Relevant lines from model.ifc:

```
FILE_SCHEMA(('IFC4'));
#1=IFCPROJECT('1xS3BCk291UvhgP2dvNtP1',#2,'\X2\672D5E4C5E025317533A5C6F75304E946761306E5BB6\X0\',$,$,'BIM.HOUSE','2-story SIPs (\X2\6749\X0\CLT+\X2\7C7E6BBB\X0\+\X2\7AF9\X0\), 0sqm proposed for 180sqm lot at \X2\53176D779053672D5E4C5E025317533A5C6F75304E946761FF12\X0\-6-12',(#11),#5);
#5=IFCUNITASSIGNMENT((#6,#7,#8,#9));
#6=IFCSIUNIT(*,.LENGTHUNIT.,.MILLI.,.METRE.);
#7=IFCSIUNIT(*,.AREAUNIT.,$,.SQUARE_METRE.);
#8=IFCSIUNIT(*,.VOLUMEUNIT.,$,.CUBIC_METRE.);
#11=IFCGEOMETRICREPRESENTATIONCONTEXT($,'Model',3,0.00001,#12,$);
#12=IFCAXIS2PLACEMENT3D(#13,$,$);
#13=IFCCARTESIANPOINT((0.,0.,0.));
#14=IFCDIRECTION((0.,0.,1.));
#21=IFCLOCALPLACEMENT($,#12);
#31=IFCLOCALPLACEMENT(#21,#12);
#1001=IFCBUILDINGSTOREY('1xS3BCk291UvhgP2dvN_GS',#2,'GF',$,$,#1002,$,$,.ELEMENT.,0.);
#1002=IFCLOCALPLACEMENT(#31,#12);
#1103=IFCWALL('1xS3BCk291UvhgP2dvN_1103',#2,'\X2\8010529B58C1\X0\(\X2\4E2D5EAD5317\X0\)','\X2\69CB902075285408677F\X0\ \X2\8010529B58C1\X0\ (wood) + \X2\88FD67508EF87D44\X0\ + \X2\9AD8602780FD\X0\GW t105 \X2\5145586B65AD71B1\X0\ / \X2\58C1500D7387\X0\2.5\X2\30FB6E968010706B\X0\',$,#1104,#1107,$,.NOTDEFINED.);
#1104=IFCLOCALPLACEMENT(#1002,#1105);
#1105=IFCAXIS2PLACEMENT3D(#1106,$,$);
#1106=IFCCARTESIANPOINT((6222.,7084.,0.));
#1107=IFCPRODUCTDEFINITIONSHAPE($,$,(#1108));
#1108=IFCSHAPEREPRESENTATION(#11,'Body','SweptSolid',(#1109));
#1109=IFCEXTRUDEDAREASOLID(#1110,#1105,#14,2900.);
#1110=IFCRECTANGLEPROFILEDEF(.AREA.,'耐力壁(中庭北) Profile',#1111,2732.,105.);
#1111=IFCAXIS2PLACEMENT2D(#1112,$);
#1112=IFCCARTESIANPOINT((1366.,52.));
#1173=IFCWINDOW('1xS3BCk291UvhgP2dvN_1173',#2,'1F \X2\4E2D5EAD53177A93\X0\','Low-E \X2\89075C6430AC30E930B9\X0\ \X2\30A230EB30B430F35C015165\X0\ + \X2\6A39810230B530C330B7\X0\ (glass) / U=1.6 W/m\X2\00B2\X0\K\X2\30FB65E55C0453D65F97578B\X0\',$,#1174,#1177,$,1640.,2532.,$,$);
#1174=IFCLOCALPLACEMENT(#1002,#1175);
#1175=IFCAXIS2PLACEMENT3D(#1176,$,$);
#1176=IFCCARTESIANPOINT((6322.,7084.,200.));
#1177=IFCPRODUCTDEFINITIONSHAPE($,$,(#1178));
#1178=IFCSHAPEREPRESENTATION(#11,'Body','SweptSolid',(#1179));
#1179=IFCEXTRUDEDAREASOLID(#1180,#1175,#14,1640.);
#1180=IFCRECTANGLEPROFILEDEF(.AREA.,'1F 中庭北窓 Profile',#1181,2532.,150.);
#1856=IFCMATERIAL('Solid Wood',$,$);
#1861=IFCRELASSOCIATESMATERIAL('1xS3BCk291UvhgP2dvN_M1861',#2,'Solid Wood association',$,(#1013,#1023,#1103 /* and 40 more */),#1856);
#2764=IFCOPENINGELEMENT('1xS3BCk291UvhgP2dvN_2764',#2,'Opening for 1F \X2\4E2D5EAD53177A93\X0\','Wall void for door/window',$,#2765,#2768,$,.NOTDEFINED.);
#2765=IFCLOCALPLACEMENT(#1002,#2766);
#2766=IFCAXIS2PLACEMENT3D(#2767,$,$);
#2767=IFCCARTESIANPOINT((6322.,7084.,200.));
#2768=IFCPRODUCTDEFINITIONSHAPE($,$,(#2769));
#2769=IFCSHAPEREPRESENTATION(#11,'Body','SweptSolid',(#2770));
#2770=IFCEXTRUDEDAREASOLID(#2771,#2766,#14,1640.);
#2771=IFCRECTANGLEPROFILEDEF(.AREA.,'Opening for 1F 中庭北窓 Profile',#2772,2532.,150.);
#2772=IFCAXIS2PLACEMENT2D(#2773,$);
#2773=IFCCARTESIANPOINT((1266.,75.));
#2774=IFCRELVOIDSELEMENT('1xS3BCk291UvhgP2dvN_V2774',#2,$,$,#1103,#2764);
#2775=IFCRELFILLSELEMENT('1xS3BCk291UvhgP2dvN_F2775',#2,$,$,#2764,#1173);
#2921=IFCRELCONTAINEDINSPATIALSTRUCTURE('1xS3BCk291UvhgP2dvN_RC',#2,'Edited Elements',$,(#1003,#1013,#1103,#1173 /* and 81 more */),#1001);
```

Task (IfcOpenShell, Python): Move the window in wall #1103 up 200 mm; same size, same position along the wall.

```python
import numpy as np
import ifcopenshell
import ifcopenshell.api.geometry
import ifcopenshell.util.placement
import ifcopenshell.util.unit

model = ifcopenshell.open("model.ifc")
unit_scale = ifcopenshell.util.unit.calculate_unit_scale(model)

window = model.by_guid("1xS3BCk291UvhgP2dvN_1173")
opening = window.FillsVoids[0].RelatingOpeningElement
dz = 0.2 / unit_scale

shift = np.array([0.0, 0.0, dz])
# The window is not placed relative to its opening, so move both.
for product in (opening, window):
    matrix = ifcopenshell.util.placement.get_local_placement(product.ObjectPlacement)
    matrix[:3, 3] += shift
    ifcopenshell.api.geometry.edit_object_placement(model, product=product, matrix=matrix, is_si=False)

print(f"moved by {dz * unit_scale:+.3f} m")

model.write("model-out.ifc")
```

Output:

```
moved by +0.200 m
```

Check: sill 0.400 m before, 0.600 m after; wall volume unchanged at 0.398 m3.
